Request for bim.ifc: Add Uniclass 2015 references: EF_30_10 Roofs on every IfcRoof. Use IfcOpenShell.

First a look at what the model holds.

```python
import ifcopenshell

model = ifcopenshell.open("bim.ifc")
print(model.schema)
print("classifications:", [c.Name for c in model.by_type("IfcClassification")])
for ifc_class in ("IfcDoor", "IfcRoof", "IfcStair", "IfcWall", "IfcWindow"):
    print(ifc_class, len(model.by_type(ifc_class)))
```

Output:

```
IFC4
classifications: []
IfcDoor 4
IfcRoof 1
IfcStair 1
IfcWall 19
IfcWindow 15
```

```python
import ifcopenshell
import ifcopenshell.api.classification

model = ifcopenshell.open("bim.ifc")

system = ifcopenshell.api.classification.add_classification(model, classification="Uniclass 2015")

codes = {
    "IfcRoof": ("EF_30_10", "Roofs"),
}
for ifc_class, (code, name) in codes.items():
    products = model.by_type(ifc_class)
    ifcopenshell.api.classification.add_reference(
        model, products=products, classification=system, identification=code, name=name
    )
    print(code, len(products))

model.write("bim_rev.ifc")
```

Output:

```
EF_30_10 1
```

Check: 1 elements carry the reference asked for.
